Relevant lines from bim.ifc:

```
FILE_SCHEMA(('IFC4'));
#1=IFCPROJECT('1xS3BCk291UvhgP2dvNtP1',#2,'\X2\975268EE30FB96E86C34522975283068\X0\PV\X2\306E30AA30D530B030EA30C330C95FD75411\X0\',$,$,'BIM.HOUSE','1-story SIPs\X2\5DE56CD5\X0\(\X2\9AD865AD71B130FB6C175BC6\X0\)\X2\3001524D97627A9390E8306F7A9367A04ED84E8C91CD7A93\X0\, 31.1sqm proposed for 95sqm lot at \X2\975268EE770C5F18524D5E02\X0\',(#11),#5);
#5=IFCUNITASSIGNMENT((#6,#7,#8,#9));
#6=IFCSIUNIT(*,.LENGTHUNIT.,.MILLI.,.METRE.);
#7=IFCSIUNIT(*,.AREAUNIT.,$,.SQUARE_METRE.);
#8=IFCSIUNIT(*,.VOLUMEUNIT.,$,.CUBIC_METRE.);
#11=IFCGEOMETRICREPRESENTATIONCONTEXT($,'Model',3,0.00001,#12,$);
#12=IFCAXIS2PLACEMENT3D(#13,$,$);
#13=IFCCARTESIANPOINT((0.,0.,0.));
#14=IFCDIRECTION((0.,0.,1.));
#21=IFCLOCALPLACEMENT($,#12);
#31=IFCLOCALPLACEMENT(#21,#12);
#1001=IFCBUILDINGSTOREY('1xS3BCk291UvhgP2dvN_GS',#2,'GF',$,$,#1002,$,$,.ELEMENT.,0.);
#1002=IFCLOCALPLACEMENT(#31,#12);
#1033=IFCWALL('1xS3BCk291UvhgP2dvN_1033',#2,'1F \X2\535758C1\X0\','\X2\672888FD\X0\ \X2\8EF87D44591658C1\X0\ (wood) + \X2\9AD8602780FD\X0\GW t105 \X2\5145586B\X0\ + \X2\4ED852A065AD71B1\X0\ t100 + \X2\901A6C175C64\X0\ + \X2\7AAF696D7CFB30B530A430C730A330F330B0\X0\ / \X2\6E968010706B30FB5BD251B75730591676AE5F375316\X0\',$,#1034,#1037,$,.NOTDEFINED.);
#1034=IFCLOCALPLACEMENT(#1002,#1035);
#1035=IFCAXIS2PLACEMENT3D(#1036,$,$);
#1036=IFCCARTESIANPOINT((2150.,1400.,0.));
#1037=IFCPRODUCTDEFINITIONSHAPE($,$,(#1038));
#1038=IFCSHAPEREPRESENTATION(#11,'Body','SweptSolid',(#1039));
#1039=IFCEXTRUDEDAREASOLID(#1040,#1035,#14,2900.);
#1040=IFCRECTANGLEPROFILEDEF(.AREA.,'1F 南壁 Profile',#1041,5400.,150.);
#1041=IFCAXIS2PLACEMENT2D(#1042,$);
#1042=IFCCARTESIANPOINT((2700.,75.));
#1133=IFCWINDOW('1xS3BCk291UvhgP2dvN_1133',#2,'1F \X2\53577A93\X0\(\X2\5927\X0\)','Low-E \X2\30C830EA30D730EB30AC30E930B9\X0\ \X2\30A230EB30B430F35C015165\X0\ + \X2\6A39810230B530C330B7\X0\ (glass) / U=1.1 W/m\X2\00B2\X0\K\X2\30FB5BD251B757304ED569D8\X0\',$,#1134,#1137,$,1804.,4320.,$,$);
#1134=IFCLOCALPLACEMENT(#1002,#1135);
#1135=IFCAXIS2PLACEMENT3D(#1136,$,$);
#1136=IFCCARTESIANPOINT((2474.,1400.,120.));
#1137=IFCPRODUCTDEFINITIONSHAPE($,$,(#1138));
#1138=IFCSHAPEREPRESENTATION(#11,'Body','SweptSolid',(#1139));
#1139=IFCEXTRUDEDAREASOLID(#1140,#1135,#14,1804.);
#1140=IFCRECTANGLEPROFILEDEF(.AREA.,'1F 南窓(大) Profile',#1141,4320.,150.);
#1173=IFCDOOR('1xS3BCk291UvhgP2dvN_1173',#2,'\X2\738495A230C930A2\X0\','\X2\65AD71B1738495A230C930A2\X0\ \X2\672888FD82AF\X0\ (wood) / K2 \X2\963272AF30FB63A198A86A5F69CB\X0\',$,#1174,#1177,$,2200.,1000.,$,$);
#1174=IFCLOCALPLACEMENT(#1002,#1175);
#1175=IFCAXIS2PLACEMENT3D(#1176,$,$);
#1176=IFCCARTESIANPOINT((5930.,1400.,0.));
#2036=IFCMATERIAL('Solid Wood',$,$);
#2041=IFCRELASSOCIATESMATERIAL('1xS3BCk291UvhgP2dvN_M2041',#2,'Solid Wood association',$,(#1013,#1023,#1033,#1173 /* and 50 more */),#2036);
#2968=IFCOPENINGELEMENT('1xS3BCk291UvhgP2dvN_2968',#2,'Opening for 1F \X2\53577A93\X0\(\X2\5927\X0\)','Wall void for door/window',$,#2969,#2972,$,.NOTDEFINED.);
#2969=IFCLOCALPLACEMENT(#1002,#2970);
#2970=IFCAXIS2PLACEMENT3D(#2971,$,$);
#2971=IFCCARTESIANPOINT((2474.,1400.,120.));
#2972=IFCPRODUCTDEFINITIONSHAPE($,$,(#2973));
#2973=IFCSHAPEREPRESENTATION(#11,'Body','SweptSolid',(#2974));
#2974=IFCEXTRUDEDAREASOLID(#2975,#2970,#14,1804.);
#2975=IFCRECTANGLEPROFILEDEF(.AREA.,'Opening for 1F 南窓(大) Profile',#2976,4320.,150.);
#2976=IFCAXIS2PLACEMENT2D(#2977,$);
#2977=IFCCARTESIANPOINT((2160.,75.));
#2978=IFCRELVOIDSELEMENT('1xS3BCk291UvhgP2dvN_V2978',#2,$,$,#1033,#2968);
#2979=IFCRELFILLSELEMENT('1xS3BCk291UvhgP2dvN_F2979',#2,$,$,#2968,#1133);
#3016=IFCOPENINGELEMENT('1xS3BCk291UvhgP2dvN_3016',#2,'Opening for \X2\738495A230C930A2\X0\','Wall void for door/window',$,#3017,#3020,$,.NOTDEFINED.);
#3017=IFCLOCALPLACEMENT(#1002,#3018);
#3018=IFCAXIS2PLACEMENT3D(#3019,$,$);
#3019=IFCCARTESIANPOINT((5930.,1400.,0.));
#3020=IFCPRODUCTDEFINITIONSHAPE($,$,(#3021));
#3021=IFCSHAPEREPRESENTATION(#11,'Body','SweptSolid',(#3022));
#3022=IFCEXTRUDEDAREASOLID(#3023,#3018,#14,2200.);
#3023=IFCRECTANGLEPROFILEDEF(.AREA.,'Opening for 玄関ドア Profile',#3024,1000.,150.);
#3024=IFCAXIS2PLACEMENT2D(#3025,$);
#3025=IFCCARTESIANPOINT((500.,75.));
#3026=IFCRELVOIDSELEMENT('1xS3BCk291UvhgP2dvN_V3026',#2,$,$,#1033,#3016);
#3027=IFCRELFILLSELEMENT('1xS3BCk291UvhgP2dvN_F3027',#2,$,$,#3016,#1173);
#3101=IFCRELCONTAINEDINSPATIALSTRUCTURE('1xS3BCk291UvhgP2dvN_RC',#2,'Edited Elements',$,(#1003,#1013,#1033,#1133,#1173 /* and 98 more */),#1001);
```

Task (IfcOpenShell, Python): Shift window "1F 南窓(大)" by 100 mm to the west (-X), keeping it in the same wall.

```python
import ifcopenshell
import ifcopenshell.api.geometry
import ifcopenshell.util.placement
import ifcopenshell.util.unit

model = ifcopenshell.open("bim.ifc")
unit_scale = ifcopenshell.util.unit.calculate_unit_scale(model)

window = model.by_id(1133)
opening = window.FillsVoids[0].RelatingOpeningElement
wall = opening.VoidsElements[0].RelatingBuildingElement

wall_matrix = ifcopenshell.util.placement.get_local_placement(wall.ObjectPlacement)
shift = wall_matrix[:3, 0] * -0.1 / unit_scale
before = ifcopenshell.util.placement.get_local_placement(window.ObjectPlacement)[:3, 3].copy()

# The window is not placed relative to its opening, so move both.
for product in (opening, window):
    matrix = ifcopenshell.util.placement.get_local_placement(product.ObjectPlacement)
    matrix[:3, 3] += shift
    ifcopenshell.api.geometry.edit_object_placement(model, product=product, matrix=matrix, is_si=False)

after = ifcopenshell.util.placement.get_local_placement(window.ObjectPlacement)[:3, 3]
print("window moved by", (after - before).round(3) + 0.0)

model.write("bim_v2.ifc")
```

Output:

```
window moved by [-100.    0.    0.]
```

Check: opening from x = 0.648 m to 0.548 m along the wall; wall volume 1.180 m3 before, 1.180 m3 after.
